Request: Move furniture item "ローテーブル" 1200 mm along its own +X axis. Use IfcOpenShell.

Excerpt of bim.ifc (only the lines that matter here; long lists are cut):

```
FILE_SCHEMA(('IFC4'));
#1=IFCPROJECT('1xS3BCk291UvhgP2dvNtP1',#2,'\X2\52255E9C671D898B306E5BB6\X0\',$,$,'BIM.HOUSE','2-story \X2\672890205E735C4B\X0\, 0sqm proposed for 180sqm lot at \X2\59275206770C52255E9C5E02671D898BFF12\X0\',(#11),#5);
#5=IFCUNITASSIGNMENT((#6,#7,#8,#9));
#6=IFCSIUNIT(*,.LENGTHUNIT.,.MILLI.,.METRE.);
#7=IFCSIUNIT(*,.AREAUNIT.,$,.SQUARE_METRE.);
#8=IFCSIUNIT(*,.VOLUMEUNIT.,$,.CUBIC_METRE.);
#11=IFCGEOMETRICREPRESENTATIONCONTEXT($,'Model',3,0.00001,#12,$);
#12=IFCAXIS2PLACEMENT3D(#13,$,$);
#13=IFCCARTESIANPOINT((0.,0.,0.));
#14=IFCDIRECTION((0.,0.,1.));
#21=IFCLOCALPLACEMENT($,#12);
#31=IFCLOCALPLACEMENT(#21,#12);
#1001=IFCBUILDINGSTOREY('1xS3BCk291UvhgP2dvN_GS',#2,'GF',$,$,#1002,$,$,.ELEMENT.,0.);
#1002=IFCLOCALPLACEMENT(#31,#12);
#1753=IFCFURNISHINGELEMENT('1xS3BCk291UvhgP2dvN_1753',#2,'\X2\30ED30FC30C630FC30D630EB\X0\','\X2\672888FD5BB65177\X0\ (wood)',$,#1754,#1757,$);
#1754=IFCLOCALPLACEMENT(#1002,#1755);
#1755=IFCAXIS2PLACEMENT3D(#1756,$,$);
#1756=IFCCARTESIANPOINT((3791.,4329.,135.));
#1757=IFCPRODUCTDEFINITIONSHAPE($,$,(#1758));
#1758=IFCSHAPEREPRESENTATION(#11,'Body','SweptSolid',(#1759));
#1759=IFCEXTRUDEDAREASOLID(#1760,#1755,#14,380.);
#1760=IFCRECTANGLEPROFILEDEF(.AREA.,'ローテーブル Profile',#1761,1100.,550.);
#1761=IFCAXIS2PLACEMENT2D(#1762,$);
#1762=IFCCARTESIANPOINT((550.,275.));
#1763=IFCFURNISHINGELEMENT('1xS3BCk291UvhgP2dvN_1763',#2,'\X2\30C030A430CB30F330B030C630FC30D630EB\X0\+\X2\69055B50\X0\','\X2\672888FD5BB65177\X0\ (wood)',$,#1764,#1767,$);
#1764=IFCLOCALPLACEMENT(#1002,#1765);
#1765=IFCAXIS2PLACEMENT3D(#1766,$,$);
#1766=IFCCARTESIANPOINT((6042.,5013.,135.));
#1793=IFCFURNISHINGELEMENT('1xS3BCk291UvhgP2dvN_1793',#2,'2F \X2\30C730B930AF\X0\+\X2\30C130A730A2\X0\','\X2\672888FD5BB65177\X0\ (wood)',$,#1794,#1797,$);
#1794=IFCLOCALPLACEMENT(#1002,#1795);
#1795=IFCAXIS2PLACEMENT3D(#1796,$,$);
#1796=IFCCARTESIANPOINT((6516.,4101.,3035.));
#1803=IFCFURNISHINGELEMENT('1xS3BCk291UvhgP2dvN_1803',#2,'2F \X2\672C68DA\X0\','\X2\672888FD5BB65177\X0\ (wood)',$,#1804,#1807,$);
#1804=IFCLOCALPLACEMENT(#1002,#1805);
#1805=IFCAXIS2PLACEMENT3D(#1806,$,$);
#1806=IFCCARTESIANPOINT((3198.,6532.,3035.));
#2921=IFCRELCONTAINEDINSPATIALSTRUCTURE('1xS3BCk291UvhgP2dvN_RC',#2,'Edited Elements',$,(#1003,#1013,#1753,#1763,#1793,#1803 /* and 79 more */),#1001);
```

```python
import ifcopenshell
import ifcopenshell.api.geometry
import ifcopenshell.util.placement

model = ifcopenshell.open("bim.ifc")

item = model.by_guid("1xS3BCk291UvhgP2dvN_1753")
matrix = ifcopenshell.util.placement.get_local_placement(item.ObjectPlacement)
matrix[:3, 3] += matrix[:3, 0] * 1200.0
ifcopenshell.api.geometry.edit_object_placement(model, product=item, matrix=matrix, is_si=False)

print(ifcopenshell.util.placement.get_local_placement(item.ObjectPlacement).round(3) + 0.0)

model.write("bim_v2.ifc")
```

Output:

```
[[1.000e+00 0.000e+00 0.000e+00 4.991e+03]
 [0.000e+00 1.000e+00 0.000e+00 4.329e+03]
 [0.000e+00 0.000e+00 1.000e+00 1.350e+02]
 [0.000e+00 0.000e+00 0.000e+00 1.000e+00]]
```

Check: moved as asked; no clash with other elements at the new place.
